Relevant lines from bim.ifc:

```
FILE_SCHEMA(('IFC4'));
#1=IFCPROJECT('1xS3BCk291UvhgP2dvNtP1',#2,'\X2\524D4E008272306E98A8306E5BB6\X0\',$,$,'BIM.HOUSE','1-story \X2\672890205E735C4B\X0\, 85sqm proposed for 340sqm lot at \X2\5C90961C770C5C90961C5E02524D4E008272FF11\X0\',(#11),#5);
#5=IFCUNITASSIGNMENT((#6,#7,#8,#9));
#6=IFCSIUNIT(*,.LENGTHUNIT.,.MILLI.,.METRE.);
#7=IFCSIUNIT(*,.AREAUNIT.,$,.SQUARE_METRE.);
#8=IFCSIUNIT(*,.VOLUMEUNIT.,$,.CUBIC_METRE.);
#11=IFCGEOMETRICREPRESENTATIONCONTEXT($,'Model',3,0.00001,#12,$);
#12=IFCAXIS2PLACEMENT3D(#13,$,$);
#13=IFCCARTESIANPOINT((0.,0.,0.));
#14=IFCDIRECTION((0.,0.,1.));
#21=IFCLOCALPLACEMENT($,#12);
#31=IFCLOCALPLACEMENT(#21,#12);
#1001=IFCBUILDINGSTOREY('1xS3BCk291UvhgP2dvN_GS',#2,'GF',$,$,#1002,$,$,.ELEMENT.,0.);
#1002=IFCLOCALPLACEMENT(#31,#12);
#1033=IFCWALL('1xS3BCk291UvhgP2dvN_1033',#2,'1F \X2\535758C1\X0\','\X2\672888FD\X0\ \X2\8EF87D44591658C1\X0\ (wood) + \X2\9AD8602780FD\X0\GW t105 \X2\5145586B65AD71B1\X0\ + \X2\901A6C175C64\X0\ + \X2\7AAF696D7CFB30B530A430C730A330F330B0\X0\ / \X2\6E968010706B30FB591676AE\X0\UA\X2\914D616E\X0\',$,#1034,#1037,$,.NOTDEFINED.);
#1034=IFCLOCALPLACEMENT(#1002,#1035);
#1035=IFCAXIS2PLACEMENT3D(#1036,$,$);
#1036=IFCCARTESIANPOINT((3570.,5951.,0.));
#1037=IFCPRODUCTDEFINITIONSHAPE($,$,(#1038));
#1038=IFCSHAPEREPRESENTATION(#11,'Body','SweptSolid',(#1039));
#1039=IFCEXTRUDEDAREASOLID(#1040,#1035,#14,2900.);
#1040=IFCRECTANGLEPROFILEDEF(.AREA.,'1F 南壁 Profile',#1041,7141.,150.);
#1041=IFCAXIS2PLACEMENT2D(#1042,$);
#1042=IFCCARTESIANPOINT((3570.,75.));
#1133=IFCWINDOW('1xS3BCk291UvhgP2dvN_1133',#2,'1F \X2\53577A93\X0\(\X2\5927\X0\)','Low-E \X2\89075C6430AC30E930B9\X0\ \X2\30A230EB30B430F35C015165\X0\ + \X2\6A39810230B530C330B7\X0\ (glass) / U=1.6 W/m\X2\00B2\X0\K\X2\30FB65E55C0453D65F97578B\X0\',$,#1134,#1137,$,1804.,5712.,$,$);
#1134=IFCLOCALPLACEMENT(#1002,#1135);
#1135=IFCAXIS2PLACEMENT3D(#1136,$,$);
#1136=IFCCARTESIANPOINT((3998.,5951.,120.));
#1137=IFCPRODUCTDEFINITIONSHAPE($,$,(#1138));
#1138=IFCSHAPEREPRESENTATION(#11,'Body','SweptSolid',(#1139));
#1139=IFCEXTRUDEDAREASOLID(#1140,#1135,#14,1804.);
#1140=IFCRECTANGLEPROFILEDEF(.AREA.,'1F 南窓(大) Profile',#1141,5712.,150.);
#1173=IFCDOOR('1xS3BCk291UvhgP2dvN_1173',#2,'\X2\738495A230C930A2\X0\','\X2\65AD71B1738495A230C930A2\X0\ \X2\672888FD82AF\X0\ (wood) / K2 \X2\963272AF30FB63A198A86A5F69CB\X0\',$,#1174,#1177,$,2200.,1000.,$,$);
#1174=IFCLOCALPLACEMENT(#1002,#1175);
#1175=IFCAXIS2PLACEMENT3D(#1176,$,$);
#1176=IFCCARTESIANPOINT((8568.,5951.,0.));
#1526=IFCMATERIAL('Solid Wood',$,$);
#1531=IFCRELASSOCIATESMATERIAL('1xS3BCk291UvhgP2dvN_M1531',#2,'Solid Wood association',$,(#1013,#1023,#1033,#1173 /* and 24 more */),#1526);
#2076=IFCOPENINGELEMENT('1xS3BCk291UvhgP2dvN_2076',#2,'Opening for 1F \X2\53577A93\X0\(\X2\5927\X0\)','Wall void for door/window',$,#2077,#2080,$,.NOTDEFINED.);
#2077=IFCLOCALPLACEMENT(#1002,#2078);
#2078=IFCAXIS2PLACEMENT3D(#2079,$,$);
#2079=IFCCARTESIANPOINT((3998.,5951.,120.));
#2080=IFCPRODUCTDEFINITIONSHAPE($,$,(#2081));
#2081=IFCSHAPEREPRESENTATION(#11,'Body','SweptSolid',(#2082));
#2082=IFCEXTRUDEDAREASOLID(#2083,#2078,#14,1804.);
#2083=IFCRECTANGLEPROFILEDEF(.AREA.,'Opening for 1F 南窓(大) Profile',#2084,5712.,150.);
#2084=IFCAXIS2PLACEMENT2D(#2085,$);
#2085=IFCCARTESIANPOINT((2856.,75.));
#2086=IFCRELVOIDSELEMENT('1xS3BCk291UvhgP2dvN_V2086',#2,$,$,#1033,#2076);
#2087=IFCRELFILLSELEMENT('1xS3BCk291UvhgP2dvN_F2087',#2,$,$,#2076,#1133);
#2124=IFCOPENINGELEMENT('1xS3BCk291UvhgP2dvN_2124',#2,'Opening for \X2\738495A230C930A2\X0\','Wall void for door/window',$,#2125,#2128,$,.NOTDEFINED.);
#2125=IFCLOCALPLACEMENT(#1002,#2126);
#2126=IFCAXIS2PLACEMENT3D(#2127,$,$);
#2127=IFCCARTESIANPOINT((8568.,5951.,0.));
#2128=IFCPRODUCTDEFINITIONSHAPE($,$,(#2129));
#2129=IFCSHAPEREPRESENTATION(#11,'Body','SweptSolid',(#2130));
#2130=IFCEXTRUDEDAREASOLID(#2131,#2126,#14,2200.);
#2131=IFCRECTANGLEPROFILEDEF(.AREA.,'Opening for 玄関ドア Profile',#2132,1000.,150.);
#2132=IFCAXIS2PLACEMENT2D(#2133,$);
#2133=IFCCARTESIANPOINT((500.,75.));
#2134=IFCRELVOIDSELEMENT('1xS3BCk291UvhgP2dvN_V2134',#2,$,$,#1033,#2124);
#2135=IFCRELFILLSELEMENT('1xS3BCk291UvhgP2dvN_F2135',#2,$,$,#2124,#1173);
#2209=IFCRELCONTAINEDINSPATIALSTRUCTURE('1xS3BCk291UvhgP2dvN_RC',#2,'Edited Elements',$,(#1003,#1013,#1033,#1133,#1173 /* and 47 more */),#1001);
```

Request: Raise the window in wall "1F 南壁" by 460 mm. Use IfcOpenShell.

```python
import numpy as np
import ifcopenshell
import ifcopenshell.api.geometry
import ifcopenshell.util.placement
import ifcopenshell.util.unit

model = ifcopenshell.open("bim.ifc")
unit_scale = ifcopenshell.util.unit.calculate_unit_scale(model)

window = model.by_id(1133)
opening = window.FillsVoids[0].RelatingOpeningElement
dz = 460.0

shift = np.array([0.0, 0.0, dz])
# The window is not placed relative to its opening, so move both.
for product in (opening, window):
    matrix = ifcopenshell.util.placement.get_local_placement(product.ObjectPlacement)
    matrix[:3, 3] += shift
    ifcopenshell.api.geometry.edit_object_placement(model, product=product, matrix=matrix, is_si=False)

print(f"moved by {dz * unit_scale:+.3f} m")

model.write("bim_rev.ifc")
```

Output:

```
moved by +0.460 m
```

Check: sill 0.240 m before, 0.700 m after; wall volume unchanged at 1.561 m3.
